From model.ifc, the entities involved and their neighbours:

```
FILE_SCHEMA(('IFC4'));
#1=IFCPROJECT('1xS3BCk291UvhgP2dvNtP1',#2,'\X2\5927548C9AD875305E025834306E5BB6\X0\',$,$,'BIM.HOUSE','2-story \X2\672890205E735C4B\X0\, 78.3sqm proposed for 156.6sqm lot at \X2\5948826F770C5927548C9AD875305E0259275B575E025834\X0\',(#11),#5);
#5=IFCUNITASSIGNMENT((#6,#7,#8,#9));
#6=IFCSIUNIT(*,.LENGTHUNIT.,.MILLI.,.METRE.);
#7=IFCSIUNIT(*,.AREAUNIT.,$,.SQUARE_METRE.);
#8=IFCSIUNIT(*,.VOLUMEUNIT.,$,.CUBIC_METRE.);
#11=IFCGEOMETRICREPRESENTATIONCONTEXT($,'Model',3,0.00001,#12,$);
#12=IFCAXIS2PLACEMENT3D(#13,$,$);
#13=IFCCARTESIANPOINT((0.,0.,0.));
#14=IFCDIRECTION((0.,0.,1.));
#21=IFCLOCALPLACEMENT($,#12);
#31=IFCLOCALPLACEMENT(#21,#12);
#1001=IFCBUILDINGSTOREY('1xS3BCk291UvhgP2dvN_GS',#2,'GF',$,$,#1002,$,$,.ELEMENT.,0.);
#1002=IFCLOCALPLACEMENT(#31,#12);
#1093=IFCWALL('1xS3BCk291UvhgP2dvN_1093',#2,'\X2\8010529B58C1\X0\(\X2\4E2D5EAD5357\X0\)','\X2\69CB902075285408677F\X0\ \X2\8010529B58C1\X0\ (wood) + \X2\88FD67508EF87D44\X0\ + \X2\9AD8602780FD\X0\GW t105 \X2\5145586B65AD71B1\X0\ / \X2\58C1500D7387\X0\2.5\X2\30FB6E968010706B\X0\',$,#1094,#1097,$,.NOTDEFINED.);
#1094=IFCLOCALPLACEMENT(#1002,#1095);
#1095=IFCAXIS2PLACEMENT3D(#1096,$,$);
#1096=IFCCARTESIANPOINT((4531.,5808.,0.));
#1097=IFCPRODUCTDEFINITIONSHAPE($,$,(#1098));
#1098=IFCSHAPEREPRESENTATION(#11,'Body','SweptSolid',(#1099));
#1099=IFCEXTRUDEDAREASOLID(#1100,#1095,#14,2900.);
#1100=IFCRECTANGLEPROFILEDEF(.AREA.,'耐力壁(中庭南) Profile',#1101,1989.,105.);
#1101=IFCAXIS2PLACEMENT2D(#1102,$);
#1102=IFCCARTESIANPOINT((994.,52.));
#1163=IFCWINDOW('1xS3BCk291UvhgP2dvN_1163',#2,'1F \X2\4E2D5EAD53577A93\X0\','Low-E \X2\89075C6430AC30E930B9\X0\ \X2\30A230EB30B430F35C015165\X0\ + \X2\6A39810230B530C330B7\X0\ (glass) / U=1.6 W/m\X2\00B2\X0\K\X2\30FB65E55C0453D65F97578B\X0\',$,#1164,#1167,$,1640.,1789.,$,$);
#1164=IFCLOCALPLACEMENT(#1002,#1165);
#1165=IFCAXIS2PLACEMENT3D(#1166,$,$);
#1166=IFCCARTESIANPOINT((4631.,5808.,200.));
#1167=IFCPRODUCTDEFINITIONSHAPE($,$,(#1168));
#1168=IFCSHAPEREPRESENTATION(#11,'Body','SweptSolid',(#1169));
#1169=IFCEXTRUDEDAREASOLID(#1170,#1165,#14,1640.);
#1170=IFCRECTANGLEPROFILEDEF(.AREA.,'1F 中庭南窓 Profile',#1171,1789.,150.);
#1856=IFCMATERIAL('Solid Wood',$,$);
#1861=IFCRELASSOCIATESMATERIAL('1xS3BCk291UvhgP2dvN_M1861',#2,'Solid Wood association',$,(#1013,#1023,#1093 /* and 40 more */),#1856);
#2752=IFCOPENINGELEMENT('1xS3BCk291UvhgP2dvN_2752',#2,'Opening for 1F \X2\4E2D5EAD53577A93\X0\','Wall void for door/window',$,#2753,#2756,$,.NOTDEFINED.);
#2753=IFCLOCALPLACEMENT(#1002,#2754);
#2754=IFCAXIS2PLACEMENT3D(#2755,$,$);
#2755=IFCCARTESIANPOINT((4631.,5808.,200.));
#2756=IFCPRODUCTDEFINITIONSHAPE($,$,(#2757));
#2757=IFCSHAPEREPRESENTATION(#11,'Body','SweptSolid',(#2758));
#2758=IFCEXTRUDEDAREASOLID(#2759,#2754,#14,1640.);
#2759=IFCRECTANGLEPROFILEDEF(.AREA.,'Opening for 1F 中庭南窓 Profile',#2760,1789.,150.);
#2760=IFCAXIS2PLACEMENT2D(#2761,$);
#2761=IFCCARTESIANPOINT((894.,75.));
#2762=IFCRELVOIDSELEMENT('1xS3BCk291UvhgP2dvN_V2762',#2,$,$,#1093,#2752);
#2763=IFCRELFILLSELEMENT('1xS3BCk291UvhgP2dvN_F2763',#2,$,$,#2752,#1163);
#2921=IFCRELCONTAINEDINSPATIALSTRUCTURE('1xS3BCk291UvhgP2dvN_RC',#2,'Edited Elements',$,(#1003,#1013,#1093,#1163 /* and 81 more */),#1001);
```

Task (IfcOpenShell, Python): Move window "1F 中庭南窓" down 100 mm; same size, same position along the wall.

```python
import numpy as np
import ifcopenshell
import ifcopenshell.api.geometry
import ifcopenshell.util.placement
import ifcopenshell.util.unit

model = ifcopenshell.open("model.ifc")
unit_scale = ifcopenshell.util.unit.calculate_unit_scale(model)

window = model.by_id(1163)
opening = window.FillsVoids[0].RelatingOpeningElement
dz = -0.1 / unit_scale

shift = np.array([0.0, 0.0, dz])
# The window is not placed relative to its opening, so move both.
for product in (opening, window):
    matrix = ifcopenshell.util.placement.get_local_placement(product.ObjectPlacement)
    matrix[:3, 3] += shift
    ifcopenshell.api.geometry.edit_object_placement(model, product=product, matrix=matrix, is_si=False)

print(f"moved by {dz * unit_scale:+.3f} m")

model.write("model_v2.ifc")
```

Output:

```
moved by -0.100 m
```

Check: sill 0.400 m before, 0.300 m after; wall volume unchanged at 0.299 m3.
